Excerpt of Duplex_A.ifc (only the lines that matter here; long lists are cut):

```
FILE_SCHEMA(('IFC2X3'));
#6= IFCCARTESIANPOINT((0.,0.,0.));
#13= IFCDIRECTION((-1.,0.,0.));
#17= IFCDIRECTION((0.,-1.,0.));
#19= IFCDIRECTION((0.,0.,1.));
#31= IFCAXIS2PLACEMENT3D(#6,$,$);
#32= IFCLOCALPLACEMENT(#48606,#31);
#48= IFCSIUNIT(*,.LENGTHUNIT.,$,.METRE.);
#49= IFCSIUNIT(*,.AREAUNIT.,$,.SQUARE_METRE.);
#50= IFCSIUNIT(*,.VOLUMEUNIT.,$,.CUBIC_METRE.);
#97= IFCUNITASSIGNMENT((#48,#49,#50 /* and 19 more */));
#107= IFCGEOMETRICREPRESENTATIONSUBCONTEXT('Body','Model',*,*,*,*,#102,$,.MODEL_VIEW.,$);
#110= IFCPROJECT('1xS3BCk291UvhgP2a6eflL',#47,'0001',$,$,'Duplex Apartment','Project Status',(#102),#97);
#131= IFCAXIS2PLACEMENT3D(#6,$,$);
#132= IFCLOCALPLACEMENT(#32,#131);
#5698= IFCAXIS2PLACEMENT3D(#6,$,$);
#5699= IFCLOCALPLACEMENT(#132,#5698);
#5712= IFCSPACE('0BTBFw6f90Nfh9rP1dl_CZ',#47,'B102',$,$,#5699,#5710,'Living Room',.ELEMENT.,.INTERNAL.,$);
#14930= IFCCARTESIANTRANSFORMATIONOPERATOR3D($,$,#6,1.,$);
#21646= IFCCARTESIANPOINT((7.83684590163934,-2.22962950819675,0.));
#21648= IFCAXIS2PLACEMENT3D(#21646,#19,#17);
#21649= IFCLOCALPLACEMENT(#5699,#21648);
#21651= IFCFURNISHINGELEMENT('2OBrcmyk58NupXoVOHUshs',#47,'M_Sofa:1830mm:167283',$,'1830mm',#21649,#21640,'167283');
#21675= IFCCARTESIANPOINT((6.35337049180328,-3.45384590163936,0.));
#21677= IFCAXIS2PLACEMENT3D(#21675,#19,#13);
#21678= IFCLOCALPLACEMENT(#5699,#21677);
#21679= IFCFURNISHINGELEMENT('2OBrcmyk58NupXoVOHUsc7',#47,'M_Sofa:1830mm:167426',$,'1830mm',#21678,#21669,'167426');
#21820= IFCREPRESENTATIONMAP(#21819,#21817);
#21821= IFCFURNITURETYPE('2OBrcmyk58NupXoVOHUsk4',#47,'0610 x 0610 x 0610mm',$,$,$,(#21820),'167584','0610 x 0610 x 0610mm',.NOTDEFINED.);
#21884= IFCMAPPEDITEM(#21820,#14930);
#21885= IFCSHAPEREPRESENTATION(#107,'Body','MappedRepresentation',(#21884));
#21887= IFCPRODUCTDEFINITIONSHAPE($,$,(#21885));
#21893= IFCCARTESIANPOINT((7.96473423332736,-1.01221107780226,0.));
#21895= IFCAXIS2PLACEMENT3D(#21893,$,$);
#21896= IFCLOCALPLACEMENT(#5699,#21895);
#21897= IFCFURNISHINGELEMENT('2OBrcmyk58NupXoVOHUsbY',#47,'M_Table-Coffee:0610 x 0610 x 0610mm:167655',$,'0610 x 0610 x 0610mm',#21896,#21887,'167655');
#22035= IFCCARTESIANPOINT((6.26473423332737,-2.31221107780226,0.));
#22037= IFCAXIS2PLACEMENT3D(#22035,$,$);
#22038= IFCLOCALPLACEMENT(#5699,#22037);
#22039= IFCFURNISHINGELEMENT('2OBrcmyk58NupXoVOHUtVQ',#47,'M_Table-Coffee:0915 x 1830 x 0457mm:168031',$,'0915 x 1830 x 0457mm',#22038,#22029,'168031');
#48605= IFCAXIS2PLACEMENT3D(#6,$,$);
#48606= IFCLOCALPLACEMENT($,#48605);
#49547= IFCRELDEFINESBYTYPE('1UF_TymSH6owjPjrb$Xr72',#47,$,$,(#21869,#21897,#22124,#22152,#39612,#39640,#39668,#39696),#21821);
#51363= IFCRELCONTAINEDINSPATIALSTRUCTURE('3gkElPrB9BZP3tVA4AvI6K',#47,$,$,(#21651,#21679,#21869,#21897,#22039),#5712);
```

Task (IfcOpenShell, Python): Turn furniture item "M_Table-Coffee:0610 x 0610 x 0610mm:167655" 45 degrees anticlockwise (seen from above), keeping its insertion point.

```python
import ifcopenshell
import ifcopenshell.api.geometry
import ifcopenshell.util.placement

model = ifcopenshell.open("Duplex_A.ifc")

item = model.by_guid("2OBrcmyk58NupXoVOHUsbY")
matrix = ifcopenshell.util.placement.get_local_placement(item.ObjectPlacement)
matrix = matrix @ ifcopenshell.util.placement.rotation(45, "Z")
ifcopenshell.api.geometry.edit_object_placement(model, product=item, matrix=matrix, is_si=False)

print(ifcopenshell.util.placement.get_local_placement(item.ObjectPlacement).round(3) + 0.0)

model.write("Duplex_A_edited.ifc")
```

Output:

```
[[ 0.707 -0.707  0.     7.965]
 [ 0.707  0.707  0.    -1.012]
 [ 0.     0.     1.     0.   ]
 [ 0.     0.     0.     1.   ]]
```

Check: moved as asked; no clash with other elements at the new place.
